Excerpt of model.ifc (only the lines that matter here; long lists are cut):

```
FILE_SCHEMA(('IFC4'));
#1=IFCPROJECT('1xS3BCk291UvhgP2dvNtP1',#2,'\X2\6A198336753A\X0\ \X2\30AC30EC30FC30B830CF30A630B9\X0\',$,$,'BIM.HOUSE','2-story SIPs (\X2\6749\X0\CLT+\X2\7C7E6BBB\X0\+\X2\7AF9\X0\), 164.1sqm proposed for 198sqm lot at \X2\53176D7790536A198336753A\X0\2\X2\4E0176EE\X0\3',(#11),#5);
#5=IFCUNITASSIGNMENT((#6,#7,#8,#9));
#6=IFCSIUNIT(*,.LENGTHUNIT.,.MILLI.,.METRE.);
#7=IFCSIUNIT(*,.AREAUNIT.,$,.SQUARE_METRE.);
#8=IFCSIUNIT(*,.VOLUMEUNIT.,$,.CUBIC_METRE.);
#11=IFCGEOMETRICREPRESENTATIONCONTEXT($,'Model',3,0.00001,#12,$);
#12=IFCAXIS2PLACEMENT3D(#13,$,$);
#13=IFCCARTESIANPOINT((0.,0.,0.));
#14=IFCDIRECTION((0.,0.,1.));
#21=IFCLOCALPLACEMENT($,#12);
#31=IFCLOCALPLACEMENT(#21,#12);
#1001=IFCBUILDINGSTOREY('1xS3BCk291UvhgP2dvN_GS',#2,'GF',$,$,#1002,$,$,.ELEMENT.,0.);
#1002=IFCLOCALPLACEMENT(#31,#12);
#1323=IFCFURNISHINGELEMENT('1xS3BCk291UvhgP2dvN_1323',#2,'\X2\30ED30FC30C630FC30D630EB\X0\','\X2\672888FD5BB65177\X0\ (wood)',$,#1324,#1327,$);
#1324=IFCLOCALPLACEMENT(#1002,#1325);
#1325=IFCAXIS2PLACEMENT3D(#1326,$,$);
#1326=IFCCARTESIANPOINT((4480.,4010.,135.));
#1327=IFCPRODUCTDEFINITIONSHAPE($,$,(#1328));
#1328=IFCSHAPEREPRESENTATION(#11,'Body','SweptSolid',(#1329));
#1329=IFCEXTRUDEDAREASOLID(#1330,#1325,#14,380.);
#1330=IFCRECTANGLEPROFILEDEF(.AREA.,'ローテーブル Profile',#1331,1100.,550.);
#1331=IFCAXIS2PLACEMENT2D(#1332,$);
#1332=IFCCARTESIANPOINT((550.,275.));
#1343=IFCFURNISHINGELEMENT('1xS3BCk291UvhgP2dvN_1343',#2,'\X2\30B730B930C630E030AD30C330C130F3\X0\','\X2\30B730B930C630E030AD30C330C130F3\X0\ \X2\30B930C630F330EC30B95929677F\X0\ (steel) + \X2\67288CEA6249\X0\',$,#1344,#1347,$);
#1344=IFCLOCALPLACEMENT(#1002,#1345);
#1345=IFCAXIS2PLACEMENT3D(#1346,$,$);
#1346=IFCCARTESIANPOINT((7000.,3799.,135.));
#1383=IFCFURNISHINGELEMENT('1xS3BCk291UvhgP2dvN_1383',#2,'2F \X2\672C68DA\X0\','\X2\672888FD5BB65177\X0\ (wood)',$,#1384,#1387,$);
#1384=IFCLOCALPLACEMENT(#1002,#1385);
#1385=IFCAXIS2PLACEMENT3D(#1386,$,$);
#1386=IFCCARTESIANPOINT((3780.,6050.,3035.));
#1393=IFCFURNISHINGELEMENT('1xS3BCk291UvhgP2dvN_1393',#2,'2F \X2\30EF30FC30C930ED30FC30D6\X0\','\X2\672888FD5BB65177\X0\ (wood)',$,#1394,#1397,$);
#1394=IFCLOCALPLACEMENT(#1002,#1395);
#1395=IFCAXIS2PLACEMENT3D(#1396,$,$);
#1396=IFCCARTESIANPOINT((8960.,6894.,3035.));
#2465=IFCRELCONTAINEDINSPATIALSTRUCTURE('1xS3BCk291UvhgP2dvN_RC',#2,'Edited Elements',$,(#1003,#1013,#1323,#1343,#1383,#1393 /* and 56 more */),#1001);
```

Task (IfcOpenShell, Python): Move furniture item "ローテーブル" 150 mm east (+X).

```python
import ifcopenshell
import ifcopenshell.api.geometry
import ifcopenshell.util.placement
import ifcopenshell.util.unit

model = ifcopenshell.open("model.ifc")
unit_scale = ifcopenshell.util.unit.calculate_unit_scale(model)

item = model.by_id(1323)
matrix = ifcopenshell.util.placement.get_local_placement(item.ObjectPlacement)
matrix[0, 3] += 0.15 / unit_scale
ifcopenshell.api.geometry.edit_object_placement(model, product=item, matrix=matrix, is_si=False)

print(ifcopenshell.util.placement.get_local_placement(item.ObjectPlacement).round(3) + 0.0)

model.write("model-out.ifc")
```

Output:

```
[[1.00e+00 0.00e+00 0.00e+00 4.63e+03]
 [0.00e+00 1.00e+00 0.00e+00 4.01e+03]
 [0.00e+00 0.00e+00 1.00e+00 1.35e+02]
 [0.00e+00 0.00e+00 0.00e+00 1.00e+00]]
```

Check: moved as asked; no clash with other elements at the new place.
